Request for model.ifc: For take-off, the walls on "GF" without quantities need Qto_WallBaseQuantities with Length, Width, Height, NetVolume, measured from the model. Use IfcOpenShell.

First a look at what the model holds.

```python
import ifcopenshell
import ifcopenshell.util.element
import ifcopenshell.util.unit

model = ifcopenshell.open("model.ifc")
print(model.schema)
for unit_type in ("LENGTHUNIT", "AREAUNIT", "VOLUMEUNIT"):
    print(unit_type, ifcopenshell.util.unit.calculate_unit_scale(model, unit_type))
storey = next(s for s in model.by_type("IfcBuildingStorey") if s.Name == "GF")
walls = [e for e in ifcopenshell.util.element.get_decomposition(storey) if e.is_a("IfcWall")]
for e in sorted(walls, key=lambda e: e.id()):
    print(e.id(), e.is_a(), e.Name, list(ifcopenshell.util.element.get_psets(e, qtos_only=True)), sep=" | ")
```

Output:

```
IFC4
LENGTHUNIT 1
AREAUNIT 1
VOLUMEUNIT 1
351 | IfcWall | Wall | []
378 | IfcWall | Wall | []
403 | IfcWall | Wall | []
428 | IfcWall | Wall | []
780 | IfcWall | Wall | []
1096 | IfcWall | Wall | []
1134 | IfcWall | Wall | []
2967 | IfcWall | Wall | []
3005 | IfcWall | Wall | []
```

```python
import ifcopenshell
import ifcopenshell.api.pset
import ifcopenshell.geom
import ifcopenshell.util.element
import ifcopenshell.util.shape
import ifcopenshell.util.unit

model = ifcopenshell.open("model.ifc")
unit_scale = ifcopenshell.util.unit.calculate_unit_scale(model)
volume_scale = ifcopenshell.util.unit.calculate_unit_scale(model, "VOLUMEUNIT")
settings = ifcopenshell.geom.settings()

storey = next(s for s in model.by_type("IfcBuildingStorey") if s.Name == "GF")
walls = [e for e in ifcopenshell.util.element.get_decomposition(storey) if e.is_a("IfcWall")]

for e in sorted(walls, key=lambda e: e.id()):
    if ifcopenshell.util.element.get_psets(e, qtos_only=True, should_inherit=False):
        continue
    # Geometry comes back in metres, in the element's own axes.
    shape = ifcopenshell.geom.create_shape(settings, e)
    values = {
        "Length": ifcopenshell.util.shape.get_x(shape.geometry) / unit_scale,
        "Width": ifcopenshell.util.shape.get_y(shape.geometry) / unit_scale,
        "Height": ifcopenshell.util.shape.get_z(shape.geometry) / unit_scale,
        "NetVolume": ifcopenshell.util.shape.get_volume(shape.geometry) / volume_scale,
    }
    qto = ifcopenshell.api.pset.add_qto(model, product=e, name="Qto_WallBaseQuantities")
    ifcopenshell.api.pset.edit_qto(model, qto=qto, properties=values)
    print(e.id(), {k: round(v, 3) for k, v in values.items()})

model.write("model-out.ifc")
```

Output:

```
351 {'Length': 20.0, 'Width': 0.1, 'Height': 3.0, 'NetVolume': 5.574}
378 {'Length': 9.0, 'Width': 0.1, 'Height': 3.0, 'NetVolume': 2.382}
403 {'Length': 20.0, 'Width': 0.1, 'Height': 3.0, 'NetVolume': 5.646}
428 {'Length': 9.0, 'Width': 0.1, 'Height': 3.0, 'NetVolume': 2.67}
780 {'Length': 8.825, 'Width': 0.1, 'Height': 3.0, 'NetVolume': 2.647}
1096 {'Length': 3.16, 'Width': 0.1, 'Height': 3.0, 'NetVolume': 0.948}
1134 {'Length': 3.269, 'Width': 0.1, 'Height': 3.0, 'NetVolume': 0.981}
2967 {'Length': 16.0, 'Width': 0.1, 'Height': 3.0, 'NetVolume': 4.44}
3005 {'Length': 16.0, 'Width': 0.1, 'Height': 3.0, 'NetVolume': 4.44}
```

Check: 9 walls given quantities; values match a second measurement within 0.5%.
